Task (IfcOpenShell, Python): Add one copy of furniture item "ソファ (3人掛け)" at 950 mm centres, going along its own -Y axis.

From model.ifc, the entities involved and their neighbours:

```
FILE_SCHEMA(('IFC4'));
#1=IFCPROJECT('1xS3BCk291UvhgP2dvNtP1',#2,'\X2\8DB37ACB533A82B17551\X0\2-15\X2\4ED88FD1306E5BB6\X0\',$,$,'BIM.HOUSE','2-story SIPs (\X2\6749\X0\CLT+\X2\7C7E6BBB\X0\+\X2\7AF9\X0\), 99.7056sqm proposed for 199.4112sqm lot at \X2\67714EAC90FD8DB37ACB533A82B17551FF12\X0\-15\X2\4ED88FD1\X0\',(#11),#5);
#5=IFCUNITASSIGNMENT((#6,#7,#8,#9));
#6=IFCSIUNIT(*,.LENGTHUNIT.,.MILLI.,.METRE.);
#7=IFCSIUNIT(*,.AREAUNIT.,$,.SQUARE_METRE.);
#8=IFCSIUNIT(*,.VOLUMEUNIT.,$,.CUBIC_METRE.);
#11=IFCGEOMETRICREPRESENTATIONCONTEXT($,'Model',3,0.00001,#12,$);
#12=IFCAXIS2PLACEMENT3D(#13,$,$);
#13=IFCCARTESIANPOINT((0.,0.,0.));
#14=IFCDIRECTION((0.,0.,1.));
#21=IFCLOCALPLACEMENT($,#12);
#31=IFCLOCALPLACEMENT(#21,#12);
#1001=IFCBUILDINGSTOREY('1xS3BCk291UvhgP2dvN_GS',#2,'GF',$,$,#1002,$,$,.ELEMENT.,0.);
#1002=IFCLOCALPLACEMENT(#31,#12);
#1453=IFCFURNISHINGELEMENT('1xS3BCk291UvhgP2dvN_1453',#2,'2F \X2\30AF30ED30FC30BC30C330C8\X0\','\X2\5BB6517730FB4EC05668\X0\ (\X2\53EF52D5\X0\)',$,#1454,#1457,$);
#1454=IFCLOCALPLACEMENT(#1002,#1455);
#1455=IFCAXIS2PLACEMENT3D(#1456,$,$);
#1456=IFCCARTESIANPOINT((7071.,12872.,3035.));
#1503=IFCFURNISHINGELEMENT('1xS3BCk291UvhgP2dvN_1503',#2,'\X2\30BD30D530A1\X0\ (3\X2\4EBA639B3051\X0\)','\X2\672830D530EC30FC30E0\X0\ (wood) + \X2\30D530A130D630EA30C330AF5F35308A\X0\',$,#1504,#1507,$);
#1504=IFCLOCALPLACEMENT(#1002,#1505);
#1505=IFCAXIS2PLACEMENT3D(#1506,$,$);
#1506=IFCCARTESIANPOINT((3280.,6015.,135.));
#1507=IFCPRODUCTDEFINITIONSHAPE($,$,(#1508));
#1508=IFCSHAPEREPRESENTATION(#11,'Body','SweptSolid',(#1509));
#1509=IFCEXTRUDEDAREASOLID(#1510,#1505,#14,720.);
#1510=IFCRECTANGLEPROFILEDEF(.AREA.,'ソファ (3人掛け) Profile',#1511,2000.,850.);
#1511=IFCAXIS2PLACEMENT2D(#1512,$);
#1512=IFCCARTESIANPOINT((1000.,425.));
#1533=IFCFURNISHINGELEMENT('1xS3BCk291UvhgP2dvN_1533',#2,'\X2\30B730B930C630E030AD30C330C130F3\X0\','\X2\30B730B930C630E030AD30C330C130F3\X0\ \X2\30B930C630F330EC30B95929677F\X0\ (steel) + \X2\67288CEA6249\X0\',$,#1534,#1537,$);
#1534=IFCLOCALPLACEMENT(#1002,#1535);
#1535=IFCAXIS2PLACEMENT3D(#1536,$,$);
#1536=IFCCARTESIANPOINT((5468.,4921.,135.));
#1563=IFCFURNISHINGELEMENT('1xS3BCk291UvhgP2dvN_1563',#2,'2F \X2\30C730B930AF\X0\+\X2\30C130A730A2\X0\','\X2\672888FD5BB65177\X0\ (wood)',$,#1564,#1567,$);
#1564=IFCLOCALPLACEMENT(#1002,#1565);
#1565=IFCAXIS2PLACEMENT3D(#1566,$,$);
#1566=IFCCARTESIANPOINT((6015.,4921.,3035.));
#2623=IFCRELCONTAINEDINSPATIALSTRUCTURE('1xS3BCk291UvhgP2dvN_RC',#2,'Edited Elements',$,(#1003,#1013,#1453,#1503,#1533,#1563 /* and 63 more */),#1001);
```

```python
import ifcopenshell
import ifcopenshell.api.geometry
import ifcopenshell.api.root
import ifcopenshell.util.element
import ifcopenshell.util.placement

model = ifcopenshell.open("model.ifc")


def reuse_history(source, copy):
    """copy_class also copies each property set's owner history, people and application; keep the originals."""
    for rel in copy.IsDefinedBy:
        if rel.is_a("IfcRelDefinesByProperties") and (history := rel.RelatingPropertyDefinition.OwnerHistory):
            rel.RelatingPropertyDefinition.OwnerHistory = source.OwnerHistory
            ifcopenshell.util.element.remove_deep2(model, history)


source = model.by_id(1503)
base = ifcopenshell.util.placement.get_local_placement(source.ObjectPlacement)
step = -base[:3, 1] * 950.0

for i in range(1, 2):
    copy = ifcopenshell.api.root.copy_class(model, product=source)
    copy.Representation = ifcopenshell.util.element.copy_deep(
        model, source.Representation, exclude=["IfcGeometricRepresentationContext", "IfcRepresentationMap"]
    )
    reuse_history(source, copy)
    matrix = base.copy()
    matrix[:3, 3] += i * step
    print("added at", matrix[:3, 3].round(3) + 0.0)
    ifcopenshell.api.geometry.edit_object_placement(model, product=copy, matrix=matrix, is_si=False)

model.write("model_rev.ifc")
```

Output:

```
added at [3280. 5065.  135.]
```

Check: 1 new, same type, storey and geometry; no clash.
